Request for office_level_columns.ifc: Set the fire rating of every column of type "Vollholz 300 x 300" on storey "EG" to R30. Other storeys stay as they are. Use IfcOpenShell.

First a look at what the model holds.

```python
import ifcopenshell
import ifcopenshell.util.element

model = ifcopenshell.open("office_level_columns.ifc")
print(model.schema)
storey = next(s for s in model.by_type("IfcBuildingStorey") if s.Name == "EG")
columns = [e for e in ifcopenshell.util.element.get_decomposition(storey) if e.is_a("IfcColumn")]
seen = {}
for e in columns:
    element_type = ifcopenshell.util.element.get_type(e)
    key = (element_type.Name if element_type != e and element_type else None, ifcopenshell.util.element.get_pset(e, "Pset_ColumnCommon", "FireRating"))
    seen[key] = seen.get(key, 0) + 1
for (name, value), count in sorted(seen.items(), key=str):
    print(count, "x", name, "|", value)
```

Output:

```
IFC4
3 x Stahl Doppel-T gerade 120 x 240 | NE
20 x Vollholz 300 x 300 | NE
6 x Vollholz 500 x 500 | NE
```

```python
import ifcopenshell
import ifcopenshell.api.pset
import ifcopenshell.util.element

model = ifcopenshell.open("office_level_columns.ifc")

storey = next(s for s in model.by_type("IfcBuildingStorey") if s.Name == "EG")
columns = [e for e in ifcopenshell.util.element.get_decomposition(storey) if e.is_a("IfcColumn")]

count = 0
for e in columns:
    element_type = ifcopenshell.util.element.get_type(e)
    if element_type in (None, e) or element_type.Name != "Vollholz 300 x 300":
        continue
    # add_pset returns the element's existing set when there is one.
    pset = ifcopenshell.api.pset.add_pset(model, product=e, name="Pset_ColumnCommon")
    ifcopenshell.api.pset.edit_pset(model, pset=pset, properties={"FireRating": "R30"})
    count += 1

print(count, "columns updated")

model.write("office_level_columns_rev.ifc")
```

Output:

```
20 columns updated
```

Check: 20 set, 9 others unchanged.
